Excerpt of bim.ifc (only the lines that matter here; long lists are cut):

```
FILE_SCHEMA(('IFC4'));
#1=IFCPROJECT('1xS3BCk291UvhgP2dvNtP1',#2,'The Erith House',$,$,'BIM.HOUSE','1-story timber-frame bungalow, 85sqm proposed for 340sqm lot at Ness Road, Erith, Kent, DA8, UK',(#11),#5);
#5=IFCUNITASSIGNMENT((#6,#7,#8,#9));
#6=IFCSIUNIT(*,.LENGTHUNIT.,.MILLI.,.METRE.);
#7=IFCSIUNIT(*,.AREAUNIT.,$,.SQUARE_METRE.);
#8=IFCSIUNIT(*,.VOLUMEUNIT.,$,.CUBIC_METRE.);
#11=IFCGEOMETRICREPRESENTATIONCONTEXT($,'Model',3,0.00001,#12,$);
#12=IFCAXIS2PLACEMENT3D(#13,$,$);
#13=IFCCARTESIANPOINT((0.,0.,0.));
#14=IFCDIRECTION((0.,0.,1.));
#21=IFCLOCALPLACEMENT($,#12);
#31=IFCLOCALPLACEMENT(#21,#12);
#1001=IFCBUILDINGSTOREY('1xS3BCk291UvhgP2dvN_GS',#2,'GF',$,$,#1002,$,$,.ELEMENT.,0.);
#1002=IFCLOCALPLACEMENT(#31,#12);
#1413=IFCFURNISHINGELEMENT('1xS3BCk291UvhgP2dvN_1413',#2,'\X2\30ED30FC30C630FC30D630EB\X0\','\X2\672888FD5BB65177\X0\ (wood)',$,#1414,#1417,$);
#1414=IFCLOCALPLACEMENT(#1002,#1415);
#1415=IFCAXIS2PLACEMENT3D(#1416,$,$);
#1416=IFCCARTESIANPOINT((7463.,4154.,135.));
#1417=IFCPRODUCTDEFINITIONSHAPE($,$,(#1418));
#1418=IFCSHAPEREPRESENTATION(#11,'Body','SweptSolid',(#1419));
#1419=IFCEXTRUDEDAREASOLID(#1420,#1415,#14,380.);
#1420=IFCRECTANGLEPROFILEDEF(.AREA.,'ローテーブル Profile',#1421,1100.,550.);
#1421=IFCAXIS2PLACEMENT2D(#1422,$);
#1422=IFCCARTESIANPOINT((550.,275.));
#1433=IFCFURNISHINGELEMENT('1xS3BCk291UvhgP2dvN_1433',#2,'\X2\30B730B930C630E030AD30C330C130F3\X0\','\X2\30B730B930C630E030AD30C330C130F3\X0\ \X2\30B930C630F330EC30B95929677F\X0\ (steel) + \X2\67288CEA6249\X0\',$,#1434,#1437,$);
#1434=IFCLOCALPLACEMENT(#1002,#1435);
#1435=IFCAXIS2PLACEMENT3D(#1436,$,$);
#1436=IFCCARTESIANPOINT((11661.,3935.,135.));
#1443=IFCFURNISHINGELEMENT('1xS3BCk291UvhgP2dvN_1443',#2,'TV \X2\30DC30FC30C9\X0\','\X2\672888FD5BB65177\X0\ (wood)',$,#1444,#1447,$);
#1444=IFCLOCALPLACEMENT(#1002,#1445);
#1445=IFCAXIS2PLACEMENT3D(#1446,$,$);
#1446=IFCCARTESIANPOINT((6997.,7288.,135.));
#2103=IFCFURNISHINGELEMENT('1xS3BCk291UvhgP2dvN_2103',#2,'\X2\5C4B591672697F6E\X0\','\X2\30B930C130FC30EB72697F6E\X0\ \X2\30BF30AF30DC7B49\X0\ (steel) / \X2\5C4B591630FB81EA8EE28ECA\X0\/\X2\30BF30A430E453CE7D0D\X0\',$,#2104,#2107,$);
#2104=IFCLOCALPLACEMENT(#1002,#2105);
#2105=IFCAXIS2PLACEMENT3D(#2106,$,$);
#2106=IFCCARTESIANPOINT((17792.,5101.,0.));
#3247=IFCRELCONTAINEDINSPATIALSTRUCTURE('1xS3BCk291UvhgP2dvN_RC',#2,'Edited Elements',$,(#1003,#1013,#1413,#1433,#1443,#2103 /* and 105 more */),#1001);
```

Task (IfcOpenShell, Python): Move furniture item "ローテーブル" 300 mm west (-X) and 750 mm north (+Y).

```python
import ifcopenshell
import ifcopenshell.api.geometry
import ifcopenshell.util.placement
import ifcopenshell.util.unit

model = ifcopenshell.open("bim.ifc")
unit_scale = ifcopenshell.util.unit.calculate_unit_scale(model)

item = model.by_guid("1xS3BCk291UvhgP2dvN_1413")
matrix = ifcopenshell.util.placement.get_local_placement(item.ObjectPlacement)
matrix[0, 3] -= 0.3 / unit_scale
matrix[1, 3] += 0.75 / unit_scale
ifcopenshell.api.geometry.edit_object_placement(model, product=item, matrix=matrix, is_si=False)

print(ifcopenshell.util.placement.get_local_placement(item.ObjectPlacement).round(3) + 0.0)

model.write("bim_updated.ifc")
```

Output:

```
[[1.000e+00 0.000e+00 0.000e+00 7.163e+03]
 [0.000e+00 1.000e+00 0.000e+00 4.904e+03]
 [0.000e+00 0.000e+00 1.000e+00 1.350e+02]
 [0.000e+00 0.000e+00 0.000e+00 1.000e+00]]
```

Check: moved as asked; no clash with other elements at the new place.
